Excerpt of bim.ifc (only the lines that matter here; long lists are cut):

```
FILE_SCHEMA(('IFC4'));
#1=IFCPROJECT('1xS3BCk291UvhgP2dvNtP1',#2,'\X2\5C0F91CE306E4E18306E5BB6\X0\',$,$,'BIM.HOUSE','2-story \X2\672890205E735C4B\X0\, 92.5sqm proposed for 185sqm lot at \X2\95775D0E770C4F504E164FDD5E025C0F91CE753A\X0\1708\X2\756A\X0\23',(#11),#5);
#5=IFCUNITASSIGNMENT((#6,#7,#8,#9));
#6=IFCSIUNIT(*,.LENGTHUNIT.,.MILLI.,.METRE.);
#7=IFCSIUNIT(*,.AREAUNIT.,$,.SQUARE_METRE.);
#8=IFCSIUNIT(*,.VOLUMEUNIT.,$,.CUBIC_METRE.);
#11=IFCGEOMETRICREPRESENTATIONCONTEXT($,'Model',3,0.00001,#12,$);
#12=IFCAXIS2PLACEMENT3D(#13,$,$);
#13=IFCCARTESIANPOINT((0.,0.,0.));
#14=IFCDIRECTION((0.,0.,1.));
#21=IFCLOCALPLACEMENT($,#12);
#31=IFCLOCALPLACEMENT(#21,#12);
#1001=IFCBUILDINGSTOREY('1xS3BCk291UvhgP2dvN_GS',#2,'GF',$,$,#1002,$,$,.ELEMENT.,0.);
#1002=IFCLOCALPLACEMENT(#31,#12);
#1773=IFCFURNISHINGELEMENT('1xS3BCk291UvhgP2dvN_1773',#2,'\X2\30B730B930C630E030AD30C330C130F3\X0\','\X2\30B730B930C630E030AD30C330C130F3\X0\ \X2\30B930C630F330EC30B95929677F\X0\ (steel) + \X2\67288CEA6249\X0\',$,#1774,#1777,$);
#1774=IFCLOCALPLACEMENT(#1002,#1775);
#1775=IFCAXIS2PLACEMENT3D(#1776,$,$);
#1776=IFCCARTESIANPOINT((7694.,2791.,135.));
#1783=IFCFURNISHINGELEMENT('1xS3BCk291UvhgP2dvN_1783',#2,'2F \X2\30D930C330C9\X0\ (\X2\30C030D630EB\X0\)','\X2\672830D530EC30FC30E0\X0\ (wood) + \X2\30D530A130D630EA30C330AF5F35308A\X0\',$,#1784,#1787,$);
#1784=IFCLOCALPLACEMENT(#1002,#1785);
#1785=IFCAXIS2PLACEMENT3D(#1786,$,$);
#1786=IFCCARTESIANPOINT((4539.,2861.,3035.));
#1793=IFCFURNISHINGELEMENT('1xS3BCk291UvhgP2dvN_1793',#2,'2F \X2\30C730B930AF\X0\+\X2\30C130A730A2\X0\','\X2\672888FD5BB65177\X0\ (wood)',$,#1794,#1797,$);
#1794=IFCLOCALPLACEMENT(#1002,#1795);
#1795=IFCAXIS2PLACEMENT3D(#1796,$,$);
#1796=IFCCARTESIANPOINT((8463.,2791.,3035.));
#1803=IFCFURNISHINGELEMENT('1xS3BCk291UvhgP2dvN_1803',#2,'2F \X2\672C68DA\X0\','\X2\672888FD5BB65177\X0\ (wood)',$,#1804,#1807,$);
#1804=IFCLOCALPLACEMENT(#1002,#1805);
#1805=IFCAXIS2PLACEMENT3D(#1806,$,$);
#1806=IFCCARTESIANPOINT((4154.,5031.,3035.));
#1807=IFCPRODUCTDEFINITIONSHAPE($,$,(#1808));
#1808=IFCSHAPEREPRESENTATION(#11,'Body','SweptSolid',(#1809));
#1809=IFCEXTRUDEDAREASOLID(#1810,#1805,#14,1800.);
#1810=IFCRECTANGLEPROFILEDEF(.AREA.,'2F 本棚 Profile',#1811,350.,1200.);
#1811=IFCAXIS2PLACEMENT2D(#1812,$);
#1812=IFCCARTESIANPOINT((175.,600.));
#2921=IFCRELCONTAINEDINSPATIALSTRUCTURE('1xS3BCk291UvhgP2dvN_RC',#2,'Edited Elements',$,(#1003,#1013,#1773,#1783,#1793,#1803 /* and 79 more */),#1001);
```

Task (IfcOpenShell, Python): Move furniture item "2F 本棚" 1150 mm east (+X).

```python
import ifcopenshell
import ifcopenshell.api.geometry
import ifcopenshell.util.placement
import ifcopenshell.util.unit

model = ifcopenshell.open("bim.ifc")
unit_scale = ifcopenshell.util.unit.calculate_unit_scale(model)

item = model.by_id(1803)
matrix = ifcopenshell.util.placement.get_local_placement(item.ObjectPlacement)
matrix[0, 3] += 1.15 / unit_scale
ifcopenshell.api.geometry.edit_object_placement(model, product=item, matrix=matrix, is_si=False)

print(ifcopenshell.util.placement.get_local_placement(item.ObjectPlacement).round(3) + 0.0)

model.write("bim_v2.ifc")
```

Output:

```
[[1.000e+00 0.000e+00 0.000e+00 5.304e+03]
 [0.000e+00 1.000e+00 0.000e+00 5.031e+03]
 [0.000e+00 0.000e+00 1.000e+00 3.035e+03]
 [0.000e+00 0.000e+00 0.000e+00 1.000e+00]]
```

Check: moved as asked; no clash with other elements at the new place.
